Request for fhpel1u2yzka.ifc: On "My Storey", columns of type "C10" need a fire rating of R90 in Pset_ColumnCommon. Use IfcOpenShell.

First a look at what the model holds.

```python
import ifcopenshell
import ifcopenshell.util.element

model = ifcopenshell.open("fhpel1u2yzka.ifc")
print(model.schema)
storey = next(s for s in model.by_type("IfcBuildingStorey") if s.Name == "My Storey")
columns = [e for e in ifcopenshell.util.element.get_decomposition(storey) if e.is_a("IfcColumn")]
seen = {}
for e in columns:
    element_type = ifcopenshell.util.element.get_type(e)
    key = (element_type.Name if element_type != e and element_type else None, ifcopenshell.util.element.get_pset(e, "Pset_ColumnCommon", "FireRating"))
    seen[key] = seen.get(key, 0) + 1
for (name, value), count in sorted(seen.items(), key=str):
    print(count, "x", name, "|", value)
```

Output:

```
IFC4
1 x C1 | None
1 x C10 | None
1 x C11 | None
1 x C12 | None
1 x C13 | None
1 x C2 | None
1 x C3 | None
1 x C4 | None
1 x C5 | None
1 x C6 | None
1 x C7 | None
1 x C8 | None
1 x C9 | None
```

```python
import ifcopenshell
import ifcopenshell.api.pset
import ifcopenshell.util.element

model = ifcopenshell.open("fhpel1u2yzka.ifc")

storey = next(s for s in model.by_type("IfcBuildingStorey") if s.Name == "My Storey")
columns = [e for e in ifcopenshell.util.element.get_decomposition(storey) if e.is_a("IfcColumn")]

count = 0
for e in columns:
    element_type = ifcopenshell.util.element.get_type(e)
    if element_type in (None, e) or element_type.Name != "C10":
        continue
    # add_pset returns the element's existing set when there is one.
    pset = ifcopenshell.api.pset.add_pset(model, product=e, name="Pset_ColumnCommon")
    ifcopenshell.api.pset.edit_pset(model, pset=pset, properties={"FireRating": "R90"})
    count += 1

print(count, "columns updated")

model.write("fhpel1u2yzka-out.ifc")
```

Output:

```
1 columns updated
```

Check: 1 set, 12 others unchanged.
